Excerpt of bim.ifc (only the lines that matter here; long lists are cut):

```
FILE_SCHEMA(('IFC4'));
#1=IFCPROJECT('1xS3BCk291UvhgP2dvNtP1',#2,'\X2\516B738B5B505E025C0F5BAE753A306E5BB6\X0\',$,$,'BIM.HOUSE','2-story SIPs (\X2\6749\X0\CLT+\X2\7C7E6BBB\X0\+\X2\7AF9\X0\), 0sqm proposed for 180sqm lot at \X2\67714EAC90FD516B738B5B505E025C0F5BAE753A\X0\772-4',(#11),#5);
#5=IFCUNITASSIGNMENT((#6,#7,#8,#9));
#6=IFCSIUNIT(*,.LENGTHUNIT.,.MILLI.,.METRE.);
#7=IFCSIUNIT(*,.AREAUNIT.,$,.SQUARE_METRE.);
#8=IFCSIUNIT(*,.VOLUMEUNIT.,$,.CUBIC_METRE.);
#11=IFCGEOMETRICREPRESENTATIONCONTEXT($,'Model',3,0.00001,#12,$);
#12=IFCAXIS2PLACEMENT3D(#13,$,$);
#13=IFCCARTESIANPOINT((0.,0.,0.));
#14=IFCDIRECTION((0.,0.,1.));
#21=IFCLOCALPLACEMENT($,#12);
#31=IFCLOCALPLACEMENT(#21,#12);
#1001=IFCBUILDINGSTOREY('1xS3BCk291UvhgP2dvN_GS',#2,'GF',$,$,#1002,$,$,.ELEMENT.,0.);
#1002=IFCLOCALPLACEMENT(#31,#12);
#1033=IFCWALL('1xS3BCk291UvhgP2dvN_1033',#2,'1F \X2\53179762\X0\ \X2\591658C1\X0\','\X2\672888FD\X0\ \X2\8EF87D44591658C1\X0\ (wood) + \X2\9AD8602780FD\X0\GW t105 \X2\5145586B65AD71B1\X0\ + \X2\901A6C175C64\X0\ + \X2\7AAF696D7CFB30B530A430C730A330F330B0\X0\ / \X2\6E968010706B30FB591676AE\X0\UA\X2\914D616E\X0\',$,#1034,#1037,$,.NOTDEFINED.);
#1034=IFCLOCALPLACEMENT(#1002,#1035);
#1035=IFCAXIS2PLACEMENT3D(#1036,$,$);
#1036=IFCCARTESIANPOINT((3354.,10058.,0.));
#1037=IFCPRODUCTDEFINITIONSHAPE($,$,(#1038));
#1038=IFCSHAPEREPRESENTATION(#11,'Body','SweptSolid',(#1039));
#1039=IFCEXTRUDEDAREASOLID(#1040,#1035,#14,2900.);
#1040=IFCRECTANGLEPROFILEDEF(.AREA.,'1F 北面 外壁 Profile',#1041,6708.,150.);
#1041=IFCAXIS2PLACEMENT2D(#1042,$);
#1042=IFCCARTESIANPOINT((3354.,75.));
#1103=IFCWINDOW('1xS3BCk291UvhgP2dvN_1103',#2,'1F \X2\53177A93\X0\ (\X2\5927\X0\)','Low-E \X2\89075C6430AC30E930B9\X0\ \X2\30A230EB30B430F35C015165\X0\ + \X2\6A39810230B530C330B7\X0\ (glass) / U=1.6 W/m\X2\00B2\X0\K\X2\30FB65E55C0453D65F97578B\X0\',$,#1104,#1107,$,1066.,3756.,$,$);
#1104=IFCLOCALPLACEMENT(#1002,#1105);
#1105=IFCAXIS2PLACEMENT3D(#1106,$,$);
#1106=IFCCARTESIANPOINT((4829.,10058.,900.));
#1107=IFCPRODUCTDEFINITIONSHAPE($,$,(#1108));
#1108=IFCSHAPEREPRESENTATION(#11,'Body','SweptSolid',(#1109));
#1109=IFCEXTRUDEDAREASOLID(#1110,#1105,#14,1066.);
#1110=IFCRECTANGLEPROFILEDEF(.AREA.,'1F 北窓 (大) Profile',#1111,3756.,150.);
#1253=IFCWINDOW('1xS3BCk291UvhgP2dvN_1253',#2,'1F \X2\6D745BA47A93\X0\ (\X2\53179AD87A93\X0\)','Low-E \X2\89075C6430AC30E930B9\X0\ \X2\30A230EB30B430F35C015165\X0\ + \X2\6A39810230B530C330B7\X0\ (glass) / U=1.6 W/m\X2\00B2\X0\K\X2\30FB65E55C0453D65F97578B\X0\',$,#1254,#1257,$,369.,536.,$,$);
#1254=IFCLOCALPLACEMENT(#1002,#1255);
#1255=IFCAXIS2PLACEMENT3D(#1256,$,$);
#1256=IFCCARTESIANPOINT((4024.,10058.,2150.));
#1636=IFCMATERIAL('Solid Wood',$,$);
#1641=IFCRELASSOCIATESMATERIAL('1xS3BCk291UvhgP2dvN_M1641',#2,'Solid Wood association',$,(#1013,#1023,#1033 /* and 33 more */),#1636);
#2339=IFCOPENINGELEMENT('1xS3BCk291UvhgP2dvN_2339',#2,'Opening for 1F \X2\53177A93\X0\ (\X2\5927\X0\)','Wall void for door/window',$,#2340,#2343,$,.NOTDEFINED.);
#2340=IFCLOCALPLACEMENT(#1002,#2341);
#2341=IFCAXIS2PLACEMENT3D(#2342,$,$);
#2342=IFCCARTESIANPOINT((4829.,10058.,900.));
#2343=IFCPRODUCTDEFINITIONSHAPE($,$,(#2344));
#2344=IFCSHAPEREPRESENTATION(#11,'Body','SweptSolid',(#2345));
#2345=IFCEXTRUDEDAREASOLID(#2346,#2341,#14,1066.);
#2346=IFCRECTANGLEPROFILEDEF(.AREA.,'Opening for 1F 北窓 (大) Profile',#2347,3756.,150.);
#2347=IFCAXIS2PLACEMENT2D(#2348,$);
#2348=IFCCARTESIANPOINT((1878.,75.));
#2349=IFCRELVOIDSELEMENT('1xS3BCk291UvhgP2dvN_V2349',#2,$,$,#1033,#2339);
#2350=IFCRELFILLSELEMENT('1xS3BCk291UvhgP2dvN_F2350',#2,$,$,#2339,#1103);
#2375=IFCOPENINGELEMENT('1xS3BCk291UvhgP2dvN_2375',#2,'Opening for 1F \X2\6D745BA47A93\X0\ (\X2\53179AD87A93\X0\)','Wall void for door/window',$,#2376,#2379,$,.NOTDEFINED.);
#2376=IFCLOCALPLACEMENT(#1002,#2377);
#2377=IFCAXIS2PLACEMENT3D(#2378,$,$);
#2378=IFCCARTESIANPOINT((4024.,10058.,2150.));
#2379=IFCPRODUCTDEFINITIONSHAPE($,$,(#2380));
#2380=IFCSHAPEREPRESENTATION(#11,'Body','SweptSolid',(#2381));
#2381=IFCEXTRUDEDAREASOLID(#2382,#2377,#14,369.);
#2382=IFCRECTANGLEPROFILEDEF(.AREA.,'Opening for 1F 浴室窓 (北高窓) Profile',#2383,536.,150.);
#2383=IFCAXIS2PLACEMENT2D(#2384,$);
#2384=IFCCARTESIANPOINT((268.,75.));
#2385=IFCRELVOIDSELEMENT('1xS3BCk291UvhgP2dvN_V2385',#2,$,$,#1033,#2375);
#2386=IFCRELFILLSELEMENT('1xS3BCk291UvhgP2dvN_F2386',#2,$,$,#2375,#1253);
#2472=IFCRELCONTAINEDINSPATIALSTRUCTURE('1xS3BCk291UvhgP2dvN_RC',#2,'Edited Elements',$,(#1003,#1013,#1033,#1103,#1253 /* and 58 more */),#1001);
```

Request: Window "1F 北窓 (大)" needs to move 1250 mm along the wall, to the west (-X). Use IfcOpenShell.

```python
import ifcopenshell
import ifcopenshell.api.geometry
import ifcopenshell.util.placement
import ifcopenshell.util.unit

model = ifcopenshell.open("bim.ifc")
unit_scale = ifcopenshell.util.unit.calculate_unit_scale(model)

window = model.by_id(1103)
opening = window.FillsVoids[0].RelatingOpeningElement
wall = opening.VoidsElements[0].RelatingBuildingElement

wall_matrix = ifcopenshell.util.placement.get_local_placement(wall.ObjectPlacement)
shift = wall_matrix[:3, 0] * -1.25 / unit_scale
before = ifcopenshell.util.placement.get_local_placement(window.ObjectPlacement)[:3, 3].copy()

# The window is not placed relative to its opening, so move both.
for product in (opening, window):
    matrix = ifcopenshell.util.placement.get_local_placement(product.ObjectPlacement)
    matrix[:3, 3] += shift
    ifcopenshell.api.geometry.edit_object_placement(model, product=product, matrix=matrix, is_si=False)

after = ifcopenshell.util.placement.get_local_placement(window.ObjectPlacement)[:3, 3]
print("window moved by", (after - before).round(3) + 0.0)

model.write("bim_v2.ifc")
```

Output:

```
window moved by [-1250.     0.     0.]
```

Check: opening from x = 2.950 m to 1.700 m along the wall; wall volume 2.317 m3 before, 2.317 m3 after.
